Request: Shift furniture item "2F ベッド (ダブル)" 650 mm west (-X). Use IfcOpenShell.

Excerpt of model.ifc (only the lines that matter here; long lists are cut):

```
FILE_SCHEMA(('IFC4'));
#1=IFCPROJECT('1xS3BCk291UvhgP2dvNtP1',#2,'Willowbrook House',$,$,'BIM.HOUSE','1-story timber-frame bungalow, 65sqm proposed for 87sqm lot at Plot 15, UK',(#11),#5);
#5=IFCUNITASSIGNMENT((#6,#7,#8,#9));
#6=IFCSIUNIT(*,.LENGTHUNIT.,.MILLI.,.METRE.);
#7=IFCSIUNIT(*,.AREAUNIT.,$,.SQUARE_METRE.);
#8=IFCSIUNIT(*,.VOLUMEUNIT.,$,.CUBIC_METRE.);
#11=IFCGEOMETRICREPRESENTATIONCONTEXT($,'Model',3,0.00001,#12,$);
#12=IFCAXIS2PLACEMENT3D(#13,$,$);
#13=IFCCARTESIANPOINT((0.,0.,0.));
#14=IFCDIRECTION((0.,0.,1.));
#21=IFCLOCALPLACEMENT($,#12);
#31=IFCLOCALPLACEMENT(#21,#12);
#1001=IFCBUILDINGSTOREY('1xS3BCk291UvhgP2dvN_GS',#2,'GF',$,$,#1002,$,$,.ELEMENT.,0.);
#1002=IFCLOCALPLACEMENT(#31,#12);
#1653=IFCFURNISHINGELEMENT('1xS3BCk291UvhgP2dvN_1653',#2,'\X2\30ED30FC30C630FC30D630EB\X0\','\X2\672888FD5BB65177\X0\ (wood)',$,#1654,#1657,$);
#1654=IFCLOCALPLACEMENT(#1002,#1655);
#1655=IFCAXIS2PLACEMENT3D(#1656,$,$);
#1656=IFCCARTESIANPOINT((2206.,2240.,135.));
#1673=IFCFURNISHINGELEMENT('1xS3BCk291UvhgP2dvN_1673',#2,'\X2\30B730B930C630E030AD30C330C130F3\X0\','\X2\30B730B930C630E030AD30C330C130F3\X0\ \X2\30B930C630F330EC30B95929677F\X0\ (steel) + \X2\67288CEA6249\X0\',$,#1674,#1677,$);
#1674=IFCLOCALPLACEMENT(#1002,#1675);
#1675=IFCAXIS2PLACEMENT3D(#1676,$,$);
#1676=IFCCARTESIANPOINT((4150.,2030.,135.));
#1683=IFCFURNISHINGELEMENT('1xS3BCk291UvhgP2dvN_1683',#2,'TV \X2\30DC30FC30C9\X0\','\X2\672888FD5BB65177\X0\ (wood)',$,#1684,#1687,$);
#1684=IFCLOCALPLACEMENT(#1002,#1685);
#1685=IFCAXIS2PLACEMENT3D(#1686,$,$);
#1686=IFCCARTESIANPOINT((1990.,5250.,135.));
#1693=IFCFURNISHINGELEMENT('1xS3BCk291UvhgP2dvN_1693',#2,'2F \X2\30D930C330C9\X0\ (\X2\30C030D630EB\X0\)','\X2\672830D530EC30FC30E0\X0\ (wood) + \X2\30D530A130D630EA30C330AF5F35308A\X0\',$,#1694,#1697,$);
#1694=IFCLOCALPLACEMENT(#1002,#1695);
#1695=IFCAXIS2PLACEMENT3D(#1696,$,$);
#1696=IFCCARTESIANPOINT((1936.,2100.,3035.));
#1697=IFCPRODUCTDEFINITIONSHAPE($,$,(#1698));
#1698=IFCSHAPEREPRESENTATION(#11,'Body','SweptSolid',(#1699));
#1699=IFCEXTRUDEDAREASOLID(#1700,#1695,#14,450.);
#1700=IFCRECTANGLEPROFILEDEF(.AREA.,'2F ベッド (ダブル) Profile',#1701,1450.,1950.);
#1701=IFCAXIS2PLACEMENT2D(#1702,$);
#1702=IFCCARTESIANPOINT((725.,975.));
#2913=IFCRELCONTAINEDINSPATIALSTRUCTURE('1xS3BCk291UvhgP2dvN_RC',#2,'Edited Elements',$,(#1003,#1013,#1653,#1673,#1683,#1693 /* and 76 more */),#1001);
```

```python
import ifcopenshell
import ifcopenshell.api.geometry
import ifcopenshell.util.placement

model = ifcopenshell.open("model.ifc")

item = model.by_id(1693)
matrix = ifcopenshell.util.placement.get_local_placement(item.ObjectPlacement)
matrix[0, 3] -= 650.0
ifcopenshell.api.geometry.edit_object_placement(model, product=item, matrix=matrix, is_si=False)

print(ifcopenshell.util.placement.get_local_placement(item.ObjectPlacement).round(3) + 0.0)

model.write("model_updated.ifc")
```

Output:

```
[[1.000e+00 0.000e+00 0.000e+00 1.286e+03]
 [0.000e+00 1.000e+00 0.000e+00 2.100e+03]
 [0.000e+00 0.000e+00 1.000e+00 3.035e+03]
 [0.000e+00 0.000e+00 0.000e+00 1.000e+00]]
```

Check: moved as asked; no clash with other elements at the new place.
